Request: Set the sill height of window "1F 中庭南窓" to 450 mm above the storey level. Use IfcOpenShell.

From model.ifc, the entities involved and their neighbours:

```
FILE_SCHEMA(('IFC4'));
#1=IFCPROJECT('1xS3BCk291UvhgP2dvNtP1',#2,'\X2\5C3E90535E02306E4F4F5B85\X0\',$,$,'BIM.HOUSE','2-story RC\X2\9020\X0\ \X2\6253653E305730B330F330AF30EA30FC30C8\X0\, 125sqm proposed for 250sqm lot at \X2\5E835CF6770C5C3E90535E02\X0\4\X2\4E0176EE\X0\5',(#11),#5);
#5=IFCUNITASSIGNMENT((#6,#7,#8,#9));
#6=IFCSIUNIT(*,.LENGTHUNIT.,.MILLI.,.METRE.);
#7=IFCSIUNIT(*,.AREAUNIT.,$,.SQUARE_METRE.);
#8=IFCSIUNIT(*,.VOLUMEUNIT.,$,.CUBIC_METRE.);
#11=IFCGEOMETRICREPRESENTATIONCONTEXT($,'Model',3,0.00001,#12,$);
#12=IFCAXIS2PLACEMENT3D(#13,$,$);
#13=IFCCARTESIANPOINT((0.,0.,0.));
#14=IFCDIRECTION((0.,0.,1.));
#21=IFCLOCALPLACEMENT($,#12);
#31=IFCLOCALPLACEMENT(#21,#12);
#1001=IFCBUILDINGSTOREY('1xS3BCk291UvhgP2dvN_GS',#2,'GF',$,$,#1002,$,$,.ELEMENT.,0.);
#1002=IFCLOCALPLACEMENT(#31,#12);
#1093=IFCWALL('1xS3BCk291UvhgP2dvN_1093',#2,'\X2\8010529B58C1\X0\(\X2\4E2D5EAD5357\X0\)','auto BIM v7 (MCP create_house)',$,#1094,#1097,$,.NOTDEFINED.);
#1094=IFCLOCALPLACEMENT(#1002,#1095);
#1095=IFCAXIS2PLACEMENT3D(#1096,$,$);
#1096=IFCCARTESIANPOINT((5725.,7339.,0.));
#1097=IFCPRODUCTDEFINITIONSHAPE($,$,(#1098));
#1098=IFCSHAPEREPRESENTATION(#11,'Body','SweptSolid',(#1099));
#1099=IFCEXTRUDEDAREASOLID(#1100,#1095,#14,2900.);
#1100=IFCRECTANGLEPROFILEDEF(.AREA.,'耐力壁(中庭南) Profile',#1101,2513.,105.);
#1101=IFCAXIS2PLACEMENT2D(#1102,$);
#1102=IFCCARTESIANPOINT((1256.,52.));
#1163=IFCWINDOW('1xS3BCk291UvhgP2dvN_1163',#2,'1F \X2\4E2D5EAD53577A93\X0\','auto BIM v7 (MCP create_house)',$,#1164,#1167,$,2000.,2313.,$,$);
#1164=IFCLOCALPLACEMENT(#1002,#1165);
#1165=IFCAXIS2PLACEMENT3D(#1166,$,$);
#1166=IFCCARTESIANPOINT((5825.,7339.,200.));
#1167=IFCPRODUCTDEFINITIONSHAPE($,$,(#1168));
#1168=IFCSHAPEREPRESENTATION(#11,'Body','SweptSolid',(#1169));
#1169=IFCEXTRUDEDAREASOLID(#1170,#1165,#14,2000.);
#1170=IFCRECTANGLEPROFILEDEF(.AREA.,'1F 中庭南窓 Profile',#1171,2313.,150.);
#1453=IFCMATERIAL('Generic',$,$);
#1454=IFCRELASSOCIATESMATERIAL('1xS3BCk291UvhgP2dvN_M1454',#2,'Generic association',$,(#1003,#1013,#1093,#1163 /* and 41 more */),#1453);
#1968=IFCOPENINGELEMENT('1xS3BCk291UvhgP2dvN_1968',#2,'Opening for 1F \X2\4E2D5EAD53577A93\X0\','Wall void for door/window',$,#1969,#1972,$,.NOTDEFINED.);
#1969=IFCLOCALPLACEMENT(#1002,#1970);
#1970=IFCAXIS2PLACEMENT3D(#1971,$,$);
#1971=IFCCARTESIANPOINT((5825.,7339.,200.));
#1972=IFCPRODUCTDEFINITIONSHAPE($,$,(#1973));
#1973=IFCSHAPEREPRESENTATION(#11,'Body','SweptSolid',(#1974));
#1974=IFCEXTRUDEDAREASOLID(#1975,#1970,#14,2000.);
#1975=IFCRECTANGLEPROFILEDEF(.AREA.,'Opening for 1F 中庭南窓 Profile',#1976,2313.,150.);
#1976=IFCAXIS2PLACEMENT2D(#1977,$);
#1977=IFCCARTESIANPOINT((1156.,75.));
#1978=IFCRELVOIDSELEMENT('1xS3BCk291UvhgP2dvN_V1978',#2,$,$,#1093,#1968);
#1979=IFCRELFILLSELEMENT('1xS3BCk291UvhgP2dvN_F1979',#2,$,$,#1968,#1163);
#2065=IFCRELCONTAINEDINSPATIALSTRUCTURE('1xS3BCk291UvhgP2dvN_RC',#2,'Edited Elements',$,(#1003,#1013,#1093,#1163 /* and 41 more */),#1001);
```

```python
import numpy as np
import ifcopenshell
import ifcopenshell.api.geometry
import ifcopenshell.geom
import ifcopenshell.util.element
import ifcopenshell.util.placement
import ifcopenshell.util.shape
import ifcopenshell.util.unit

model = ifcopenshell.open("model.ifc")
unit_scale = ifcopenshell.util.unit.calculate_unit_scale(model)

window = model.by_id(1163)
opening = window.FillsVoids[0].RelatingOpeningElement
storey = ifcopenshell.util.element.get_container(window, ifc_class="IfcBuildingStorey")
level = ifcopenshell.util.placement.get_local_placement(storey.ObjectPlacement)[2, 3]

# The opening's origin need not be at the sill, so measure its lowest point.
shape = ifcopenshell.geom.create_shape(ifcopenshell.geom.settings(), opening)
bottom = ifcopenshell.util.shape.get_shape_bottom_elevation(shape, shape.geometry) / unit_scale
dz = level + 0.45 / unit_scale - bottom

shift = np.array([0.0, 0.0, dz])
# The window is not placed relative to its opening, so move both.
for product in (opening, window):
    matrix = ifcopenshell.util.placement.get_local_placement(product.ObjectPlacement)
    matrix[:3, 3] += shift
    ifcopenshell.api.geometry.edit_object_placement(model, product=product, matrix=matrix, is_si=False)

print(f"moved by {dz * unit_scale:+.3f} m")

model.write("model-out.ifc")
```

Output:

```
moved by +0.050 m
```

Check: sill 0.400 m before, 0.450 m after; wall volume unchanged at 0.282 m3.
